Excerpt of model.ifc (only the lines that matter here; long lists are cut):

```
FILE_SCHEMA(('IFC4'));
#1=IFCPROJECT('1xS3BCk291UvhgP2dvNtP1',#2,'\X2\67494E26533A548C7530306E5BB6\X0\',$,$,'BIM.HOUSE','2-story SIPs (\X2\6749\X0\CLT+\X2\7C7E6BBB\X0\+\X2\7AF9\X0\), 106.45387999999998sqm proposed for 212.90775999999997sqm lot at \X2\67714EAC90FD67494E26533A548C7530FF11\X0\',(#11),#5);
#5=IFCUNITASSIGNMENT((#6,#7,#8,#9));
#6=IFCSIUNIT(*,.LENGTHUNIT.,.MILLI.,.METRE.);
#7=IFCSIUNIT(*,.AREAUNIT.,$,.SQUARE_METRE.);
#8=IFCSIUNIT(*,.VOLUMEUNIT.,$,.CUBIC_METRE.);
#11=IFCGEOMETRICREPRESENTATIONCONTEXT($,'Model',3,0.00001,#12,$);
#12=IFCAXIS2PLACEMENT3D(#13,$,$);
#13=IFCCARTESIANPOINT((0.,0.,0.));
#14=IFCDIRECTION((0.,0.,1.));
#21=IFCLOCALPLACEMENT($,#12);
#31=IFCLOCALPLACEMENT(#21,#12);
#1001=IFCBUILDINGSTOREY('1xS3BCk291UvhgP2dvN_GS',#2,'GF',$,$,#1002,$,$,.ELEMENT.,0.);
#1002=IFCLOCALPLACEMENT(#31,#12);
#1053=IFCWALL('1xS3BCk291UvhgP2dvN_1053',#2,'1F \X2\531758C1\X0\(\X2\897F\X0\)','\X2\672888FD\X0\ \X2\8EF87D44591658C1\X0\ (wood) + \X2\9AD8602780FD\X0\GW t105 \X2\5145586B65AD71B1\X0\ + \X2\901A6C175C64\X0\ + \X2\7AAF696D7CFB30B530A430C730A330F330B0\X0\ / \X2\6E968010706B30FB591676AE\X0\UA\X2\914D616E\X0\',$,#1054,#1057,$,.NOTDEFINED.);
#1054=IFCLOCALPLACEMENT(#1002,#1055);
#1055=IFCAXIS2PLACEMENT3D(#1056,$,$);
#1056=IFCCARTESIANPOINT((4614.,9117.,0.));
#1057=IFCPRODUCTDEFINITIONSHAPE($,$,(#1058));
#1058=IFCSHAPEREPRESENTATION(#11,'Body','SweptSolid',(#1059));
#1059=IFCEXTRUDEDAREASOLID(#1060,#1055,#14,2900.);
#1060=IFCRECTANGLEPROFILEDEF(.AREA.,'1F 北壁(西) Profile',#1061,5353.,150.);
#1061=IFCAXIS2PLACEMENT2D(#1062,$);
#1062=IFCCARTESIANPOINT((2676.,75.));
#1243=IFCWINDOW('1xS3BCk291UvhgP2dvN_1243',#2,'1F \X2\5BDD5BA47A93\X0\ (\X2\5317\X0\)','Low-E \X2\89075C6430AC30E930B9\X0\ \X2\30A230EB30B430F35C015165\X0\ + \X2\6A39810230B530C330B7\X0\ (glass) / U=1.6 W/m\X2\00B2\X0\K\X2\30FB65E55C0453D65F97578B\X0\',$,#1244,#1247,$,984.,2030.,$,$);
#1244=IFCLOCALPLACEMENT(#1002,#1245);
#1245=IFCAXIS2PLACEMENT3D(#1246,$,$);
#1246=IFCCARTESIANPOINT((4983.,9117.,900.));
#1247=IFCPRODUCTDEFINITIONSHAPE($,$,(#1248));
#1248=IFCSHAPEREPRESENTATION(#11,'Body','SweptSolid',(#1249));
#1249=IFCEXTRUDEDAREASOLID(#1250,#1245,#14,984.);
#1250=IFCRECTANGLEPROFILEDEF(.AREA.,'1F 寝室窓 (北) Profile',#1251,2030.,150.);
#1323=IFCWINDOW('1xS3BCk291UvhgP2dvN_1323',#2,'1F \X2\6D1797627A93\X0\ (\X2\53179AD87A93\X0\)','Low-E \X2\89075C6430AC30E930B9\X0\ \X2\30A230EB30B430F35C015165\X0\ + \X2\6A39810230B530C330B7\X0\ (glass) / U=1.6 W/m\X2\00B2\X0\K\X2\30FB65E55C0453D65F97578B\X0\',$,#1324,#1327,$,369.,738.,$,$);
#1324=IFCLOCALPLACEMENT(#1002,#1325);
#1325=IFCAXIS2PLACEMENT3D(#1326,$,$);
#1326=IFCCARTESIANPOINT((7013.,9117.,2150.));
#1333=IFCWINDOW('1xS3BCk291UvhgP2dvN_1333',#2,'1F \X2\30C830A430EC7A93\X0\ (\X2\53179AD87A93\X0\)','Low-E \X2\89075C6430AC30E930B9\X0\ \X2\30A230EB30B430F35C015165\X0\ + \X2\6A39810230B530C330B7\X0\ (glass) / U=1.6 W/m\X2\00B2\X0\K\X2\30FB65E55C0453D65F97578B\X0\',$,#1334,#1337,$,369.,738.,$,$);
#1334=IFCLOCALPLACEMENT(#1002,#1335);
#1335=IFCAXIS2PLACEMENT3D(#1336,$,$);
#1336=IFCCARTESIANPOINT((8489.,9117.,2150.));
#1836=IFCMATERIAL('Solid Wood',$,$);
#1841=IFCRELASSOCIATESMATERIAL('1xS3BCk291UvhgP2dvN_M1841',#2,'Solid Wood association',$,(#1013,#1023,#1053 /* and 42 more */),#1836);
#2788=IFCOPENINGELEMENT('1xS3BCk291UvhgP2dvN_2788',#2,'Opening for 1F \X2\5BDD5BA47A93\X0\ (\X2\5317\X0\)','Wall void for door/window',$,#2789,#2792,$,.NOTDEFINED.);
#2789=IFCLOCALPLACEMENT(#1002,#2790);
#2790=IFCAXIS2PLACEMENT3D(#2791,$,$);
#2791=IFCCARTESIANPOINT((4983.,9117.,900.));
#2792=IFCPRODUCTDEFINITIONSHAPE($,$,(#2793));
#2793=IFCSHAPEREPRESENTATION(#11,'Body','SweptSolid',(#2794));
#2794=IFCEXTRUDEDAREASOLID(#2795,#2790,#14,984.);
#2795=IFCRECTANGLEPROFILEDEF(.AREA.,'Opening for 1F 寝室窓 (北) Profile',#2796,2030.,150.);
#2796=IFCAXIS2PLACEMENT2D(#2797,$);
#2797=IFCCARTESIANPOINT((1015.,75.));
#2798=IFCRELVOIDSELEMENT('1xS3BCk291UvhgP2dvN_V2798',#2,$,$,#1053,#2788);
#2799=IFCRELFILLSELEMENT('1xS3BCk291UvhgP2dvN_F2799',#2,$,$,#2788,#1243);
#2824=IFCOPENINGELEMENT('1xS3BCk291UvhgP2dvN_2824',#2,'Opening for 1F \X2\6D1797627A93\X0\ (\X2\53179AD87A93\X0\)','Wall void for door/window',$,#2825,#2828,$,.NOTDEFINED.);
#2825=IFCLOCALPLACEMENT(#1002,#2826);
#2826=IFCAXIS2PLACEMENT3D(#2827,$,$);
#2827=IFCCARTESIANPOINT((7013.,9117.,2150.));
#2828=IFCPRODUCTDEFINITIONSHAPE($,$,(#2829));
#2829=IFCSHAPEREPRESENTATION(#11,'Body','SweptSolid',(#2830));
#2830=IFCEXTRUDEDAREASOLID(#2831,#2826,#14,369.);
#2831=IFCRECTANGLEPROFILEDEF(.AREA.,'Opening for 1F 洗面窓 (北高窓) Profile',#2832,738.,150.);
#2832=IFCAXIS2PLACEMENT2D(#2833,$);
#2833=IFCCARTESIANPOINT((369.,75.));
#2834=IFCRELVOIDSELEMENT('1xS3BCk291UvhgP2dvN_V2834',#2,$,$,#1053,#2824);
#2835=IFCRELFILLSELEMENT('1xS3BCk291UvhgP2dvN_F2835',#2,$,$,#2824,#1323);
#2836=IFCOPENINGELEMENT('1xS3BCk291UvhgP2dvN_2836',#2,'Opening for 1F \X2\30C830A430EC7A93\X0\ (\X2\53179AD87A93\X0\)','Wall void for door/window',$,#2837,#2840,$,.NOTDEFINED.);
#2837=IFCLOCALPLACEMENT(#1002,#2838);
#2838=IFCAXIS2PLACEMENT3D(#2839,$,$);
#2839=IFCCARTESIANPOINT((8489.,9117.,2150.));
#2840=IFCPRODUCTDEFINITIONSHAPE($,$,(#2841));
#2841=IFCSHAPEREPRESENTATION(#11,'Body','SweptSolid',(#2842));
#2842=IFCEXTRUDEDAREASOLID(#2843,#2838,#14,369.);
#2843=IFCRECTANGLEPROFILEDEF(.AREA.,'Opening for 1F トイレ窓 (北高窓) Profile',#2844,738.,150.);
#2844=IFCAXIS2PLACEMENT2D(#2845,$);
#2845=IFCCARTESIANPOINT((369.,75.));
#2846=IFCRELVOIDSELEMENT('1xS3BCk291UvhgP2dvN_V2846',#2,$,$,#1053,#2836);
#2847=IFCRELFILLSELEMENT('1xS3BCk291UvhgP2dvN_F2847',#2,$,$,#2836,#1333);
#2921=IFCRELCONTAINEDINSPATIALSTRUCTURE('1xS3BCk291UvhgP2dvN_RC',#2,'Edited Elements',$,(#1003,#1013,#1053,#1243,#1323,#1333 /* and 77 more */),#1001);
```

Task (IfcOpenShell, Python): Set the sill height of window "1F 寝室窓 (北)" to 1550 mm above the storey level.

```python
import numpy as np
import ifcopenshell
import ifcopenshell.api.geometry
import ifcopenshell.geom
import ifcopenshell.util.element
import ifcopenshell.util.placement
import ifcopenshell.util.shape
import ifcopenshell.util.unit

model = ifcopenshell.open("model.ifc")
unit_scale = ifcopenshell.util.unit.calculate_unit_scale(model)

window = model.by_guid("1xS3BCk291UvhgP2dvN_1243")
opening = window.FillsVoids[0].RelatingOpeningElement
storey = ifcopenshell.util.element.get_container(window, ifc_class="IfcBuildingStorey")
level = ifcopenshell.util.placement.get_local_placement(storey.ObjectPlacement)[2, 3]

# The opening's origin need not be at the sill, so measure its lowest point.
shape = ifcopenshell.geom.create_shape(ifcopenshell.geom.settings(), opening)
bottom = ifcopenshell.util.shape.get_shape_bottom_elevation(shape, shape.geometry) / unit_scale
dz = level + 1550.0 - bottom

shift = np.array([0.0, 0.0, dz])
# The window is not placed relative to its opening, so move both.
for product in (opening, window):
    matrix = ifcopenshell.util.placement.get_local_placement(product.ObjectPlacement)
    matrix[:3, 3] += shift
    ifcopenshell.api.geometry.edit_object_placement(model, product=product, matrix=matrix, is_si=False)

print(f"moved by {dz * unit_scale:+.3f} m")

model.write("model_v2.ifc")
```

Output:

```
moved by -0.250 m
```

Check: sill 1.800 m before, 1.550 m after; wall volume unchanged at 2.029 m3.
